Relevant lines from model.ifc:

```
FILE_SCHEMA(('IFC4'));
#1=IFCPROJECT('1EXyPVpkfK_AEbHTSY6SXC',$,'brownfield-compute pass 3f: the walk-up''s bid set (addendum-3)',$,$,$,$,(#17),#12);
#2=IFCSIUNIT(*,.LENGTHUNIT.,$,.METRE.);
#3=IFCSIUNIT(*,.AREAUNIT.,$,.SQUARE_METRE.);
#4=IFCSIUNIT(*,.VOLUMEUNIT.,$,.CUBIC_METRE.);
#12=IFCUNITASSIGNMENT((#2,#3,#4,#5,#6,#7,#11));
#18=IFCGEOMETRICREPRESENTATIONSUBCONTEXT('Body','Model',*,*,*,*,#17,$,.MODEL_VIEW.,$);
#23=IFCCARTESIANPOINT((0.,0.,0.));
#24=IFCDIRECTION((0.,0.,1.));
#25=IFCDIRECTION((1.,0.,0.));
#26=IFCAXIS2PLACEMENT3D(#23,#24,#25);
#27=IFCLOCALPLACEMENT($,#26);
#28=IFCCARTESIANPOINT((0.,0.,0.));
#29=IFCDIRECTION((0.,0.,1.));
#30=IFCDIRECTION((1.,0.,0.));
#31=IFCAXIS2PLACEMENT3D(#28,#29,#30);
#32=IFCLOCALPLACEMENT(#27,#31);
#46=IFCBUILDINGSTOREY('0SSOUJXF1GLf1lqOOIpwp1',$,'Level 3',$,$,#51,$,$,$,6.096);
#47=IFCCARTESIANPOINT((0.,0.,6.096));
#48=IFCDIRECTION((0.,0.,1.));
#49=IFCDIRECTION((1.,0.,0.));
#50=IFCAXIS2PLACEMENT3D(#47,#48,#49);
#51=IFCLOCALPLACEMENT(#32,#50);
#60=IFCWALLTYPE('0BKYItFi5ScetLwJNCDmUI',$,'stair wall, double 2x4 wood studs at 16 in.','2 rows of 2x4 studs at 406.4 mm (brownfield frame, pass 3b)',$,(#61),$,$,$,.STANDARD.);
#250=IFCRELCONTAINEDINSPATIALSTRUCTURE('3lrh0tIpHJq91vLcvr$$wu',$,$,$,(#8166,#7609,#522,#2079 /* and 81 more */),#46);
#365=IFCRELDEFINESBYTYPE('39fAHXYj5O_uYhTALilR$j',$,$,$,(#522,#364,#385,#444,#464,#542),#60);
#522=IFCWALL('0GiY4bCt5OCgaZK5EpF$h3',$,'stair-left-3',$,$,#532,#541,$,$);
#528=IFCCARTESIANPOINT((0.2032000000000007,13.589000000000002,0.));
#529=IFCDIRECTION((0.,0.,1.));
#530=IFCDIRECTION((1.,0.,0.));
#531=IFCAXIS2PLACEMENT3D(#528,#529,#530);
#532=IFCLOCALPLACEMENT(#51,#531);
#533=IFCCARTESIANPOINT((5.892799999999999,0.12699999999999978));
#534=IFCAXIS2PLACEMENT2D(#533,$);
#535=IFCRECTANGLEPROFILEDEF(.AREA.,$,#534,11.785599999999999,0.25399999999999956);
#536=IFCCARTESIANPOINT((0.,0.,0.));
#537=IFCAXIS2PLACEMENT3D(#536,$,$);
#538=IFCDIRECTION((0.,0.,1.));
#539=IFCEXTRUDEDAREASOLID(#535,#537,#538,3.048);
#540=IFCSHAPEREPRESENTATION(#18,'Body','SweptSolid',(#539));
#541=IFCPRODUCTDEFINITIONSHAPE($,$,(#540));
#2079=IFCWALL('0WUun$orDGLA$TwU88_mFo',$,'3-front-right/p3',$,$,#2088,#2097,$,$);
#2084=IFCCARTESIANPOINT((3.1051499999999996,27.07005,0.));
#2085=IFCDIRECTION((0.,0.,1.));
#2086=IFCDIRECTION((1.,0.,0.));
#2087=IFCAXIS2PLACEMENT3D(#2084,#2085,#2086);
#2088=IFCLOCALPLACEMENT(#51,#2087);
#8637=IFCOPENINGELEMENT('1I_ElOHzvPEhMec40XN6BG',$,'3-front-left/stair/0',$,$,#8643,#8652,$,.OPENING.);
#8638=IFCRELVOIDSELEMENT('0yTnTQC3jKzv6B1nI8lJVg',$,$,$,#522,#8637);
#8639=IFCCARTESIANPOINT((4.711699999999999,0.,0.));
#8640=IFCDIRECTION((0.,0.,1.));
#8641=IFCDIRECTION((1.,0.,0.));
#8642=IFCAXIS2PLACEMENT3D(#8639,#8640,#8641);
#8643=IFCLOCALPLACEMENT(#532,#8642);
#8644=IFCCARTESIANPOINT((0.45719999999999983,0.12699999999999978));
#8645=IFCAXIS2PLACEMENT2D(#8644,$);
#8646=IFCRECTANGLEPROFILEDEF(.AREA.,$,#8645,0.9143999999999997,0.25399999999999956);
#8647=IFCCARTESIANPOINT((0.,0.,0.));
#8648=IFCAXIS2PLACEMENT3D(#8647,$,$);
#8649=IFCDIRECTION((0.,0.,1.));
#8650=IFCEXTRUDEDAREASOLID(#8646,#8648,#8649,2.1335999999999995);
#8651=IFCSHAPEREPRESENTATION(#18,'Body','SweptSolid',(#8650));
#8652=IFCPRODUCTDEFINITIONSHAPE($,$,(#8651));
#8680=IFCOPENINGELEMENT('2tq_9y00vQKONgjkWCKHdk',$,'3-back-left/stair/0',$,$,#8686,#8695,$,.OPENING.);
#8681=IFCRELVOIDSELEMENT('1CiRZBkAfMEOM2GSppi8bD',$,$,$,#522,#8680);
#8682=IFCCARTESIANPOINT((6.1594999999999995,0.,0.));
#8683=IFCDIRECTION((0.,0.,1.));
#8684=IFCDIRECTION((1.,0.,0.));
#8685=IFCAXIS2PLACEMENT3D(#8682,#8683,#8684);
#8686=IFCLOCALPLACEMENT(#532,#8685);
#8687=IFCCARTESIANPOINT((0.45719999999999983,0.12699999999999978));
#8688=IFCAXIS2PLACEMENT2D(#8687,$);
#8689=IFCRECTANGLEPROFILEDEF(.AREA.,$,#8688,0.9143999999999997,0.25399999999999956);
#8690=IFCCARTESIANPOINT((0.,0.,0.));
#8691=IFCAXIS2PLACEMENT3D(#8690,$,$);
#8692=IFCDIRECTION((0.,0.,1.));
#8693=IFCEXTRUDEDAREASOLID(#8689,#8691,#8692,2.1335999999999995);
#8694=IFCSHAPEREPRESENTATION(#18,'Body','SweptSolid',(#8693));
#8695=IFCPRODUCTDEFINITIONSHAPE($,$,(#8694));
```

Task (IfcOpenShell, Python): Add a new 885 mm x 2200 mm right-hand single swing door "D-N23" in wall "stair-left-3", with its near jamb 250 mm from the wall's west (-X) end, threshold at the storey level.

```python
import numpy as np
import ifcopenshell
import ifcopenshell.api.feature
import ifcopenshell.api.geometry
import ifcopenshell.api.root
import ifcopenshell.api.spatial
import ifcopenshell.geom
import ifcopenshell.util.element
import ifcopenshell.util.placement
import ifcopenshell.util.representation
import ifcopenshell.util.shape
import ifcopenshell.util.unit

model = ifcopenshell.open("model.ifc")
unit_scale = ifcopenshell.util.unit.calculate_unit_scale(model)
settings = ifcopenshell.geom.settings()


def volume(element):
    """Net volume in cubic metres, openings subtracted."""
    shape = ifcopenshell.geom.create_shape(settings, element)
    return ifcopenshell.util.shape.get_volume(shape.geometry)


wall = model.by_guid("0GiY4bCt5OCgaZK5EpF$h3")
storey = ifcopenshell.util.element.get_container(wall, ifc_class="IfcBuildingStorey")
context = ifcopenshell.util.representation.get_context(model, "Model", "Body", "MODEL_VIEW")
before = volume(wall)

width, height, from_end, sill = 0.885, 2.2, 0.25, 0.0  # metres

# The wall runs along its own X axis, and the end named is its -X end.
wall_shape = ifcopenshell.geom.create_shape(settings, wall)
x, y, z = ifcopenshell.util.shape.get_vertices(wall_shape.geometry).T
start = x.min() + from_end
face, thickness = float(y.min()), float(y.max() - y.min())
wall_matrix = ifcopenshell.util.placement.get_local_placement(wall.ObjectPlacement)
level = ifcopenshell.util.placement.get_local_placement(storey.ObjectPlacement)[2, 3]


def in_wall(x, y):
    """Placement at x, y metres in the wall's axes, at sill height."""
    matrix = wall_matrix.copy()
    matrix[:, 3] = wall_matrix @ np.array([x / unit_scale, y / unit_scale, 0.0, 1.0])
    matrix[2, 3] = level + sill / unit_scale
    return matrix


# Opening: a box that overshoots both wall faces by 50 mm.
opening = ifcopenshell.api.root.create_entity(model, ifc_class="IfcOpeningElement", predefined_type="OPENING")
box = ifcopenshell.api.geometry.add_wall_representation(
    model, context=context, length=width, height=height, thickness=thickness + 0.1
)
ifcopenshell.api.geometry.assign_representation(model, product=opening, representation=box)
ifcopenshell.api.geometry.edit_object_placement(model, product=opening, matrix=in_wall(start, face - 0.05), is_si=False)
ifcopenshell.api.feature.add_feature(model, feature=opening, element=wall)

door = ifcopenshell.api.root.create_entity(model, ifc_class="IfcDoor", name="D-N23", predefined_type="DOOR")
door.OverallWidth, door.OverallHeight = width / unit_scale, height / unit_scale
door.OperationType = "SINGLE_SWING_RIGHT"
body = ifcopenshell.api.geometry.add_door_representation(
    model,
    context=context,
    overall_width=door.OverallWidth,
    overall_height=door.OverallHeight,
    operation_type="SINGLE_SWING_RIGHT",
    lining_properties={"LiningDepth": thickness / unit_scale, "ThresholdDepth": thickness / unit_scale},
)
ifcopenshell.api.geometry.assign_representation(model, product=door, representation=body)
ifcopenshell.api.spatial.assign_container(model, products=[door], relating_structure=storey)
ifcopenshell.api.feature.add_filling(model, opening=opening, element=door)

# The lining spans the wall, so the door starts at the wall face.
ifcopenshell.api.geometry.edit_object_placement(model, product=door, matrix=in_wall(start, face), is_si=False)

after = volume(wall)

print(f"wall volume {before:.3f} -> {after:.3f} m3")

model.write("model_edited.ifc")
```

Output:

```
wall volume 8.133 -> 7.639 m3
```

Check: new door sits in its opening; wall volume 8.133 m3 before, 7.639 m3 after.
